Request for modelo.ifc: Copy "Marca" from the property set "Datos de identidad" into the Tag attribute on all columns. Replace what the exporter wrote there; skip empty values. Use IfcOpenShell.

First a look at what the model holds.

```python
import ifcopenshell
import ifcopenshell.util.element

model = ifcopenshell.open("modelo.ifc")
print(model.schema)
columns = model.by_type("IfcColumn")
print(len(columns), "columns")
for e in columns[:8]:
    source = ifcopenshell.util.element.get_pset(e, "Datos de identidad", "Marca")
    target = e.Tag
    print(e.id(), repr(source), repr(target), sep=" | ")
```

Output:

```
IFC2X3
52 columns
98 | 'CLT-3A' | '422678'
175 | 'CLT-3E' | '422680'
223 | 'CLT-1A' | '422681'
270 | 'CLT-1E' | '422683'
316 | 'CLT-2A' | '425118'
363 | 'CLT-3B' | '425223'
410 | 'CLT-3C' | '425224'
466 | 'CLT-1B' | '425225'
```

```python
import ifcopenshell
import ifcopenshell.util.element

model = ifcopenshell.open("modelo.ifc")

count = 0
for e in model.by_type("IfcColumn"):
    value = ifcopenshell.util.element.get_pset(e, "Datos de identidad", "Marca")
    current = e.Tag
    if not value or not value.strip() or current == value:
        continue
    e.Tag = value
    count += 1

print(count, "columns updated")

model.write("modelo_updated.ifc")
```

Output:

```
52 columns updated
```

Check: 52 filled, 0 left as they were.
